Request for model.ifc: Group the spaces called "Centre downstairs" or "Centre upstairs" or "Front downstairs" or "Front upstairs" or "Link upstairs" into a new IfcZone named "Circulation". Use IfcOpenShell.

First a look at what the model holds.

```python
import ifcopenshell

model = ifcopenshell.open("model.ifc")
print(model.schema)
seen = {}
for space in model.by_type("IfcSpace"):
    seen[space.Name] = seen.get(space.Name, 0) + 1
for name, count in sorted(seen.items(), key=str):
    print(count, "x", name)
print("zones:", [z.Name for z in model.by_type("IfcZone")][:20])
```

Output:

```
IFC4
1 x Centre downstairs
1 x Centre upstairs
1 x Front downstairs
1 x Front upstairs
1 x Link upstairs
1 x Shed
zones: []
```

```python
import ifcopenshell
import ifcopenshell.api.group
import ifcopenshell.api.root

model = ifcopenshell.open("model.ifc")

names = {"Centre downstairs", "Centre upstairs", "Front downstairs", "Front upstairs", "Link upstairs"}
spaces = [s for s in model.by_type("IfcSpace") if s.Name in names]

zone = ifcopenshell.api.root.create_entity(model, ifc_class="IfcZone", name="Circulation")
ifcopenshell.api.group.assign_group(model, products=spaces, group=zone)
print(len(spaces), "spaces in", zone.Name)

model.write("model-out.ifc")
```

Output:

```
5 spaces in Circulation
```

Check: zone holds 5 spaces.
